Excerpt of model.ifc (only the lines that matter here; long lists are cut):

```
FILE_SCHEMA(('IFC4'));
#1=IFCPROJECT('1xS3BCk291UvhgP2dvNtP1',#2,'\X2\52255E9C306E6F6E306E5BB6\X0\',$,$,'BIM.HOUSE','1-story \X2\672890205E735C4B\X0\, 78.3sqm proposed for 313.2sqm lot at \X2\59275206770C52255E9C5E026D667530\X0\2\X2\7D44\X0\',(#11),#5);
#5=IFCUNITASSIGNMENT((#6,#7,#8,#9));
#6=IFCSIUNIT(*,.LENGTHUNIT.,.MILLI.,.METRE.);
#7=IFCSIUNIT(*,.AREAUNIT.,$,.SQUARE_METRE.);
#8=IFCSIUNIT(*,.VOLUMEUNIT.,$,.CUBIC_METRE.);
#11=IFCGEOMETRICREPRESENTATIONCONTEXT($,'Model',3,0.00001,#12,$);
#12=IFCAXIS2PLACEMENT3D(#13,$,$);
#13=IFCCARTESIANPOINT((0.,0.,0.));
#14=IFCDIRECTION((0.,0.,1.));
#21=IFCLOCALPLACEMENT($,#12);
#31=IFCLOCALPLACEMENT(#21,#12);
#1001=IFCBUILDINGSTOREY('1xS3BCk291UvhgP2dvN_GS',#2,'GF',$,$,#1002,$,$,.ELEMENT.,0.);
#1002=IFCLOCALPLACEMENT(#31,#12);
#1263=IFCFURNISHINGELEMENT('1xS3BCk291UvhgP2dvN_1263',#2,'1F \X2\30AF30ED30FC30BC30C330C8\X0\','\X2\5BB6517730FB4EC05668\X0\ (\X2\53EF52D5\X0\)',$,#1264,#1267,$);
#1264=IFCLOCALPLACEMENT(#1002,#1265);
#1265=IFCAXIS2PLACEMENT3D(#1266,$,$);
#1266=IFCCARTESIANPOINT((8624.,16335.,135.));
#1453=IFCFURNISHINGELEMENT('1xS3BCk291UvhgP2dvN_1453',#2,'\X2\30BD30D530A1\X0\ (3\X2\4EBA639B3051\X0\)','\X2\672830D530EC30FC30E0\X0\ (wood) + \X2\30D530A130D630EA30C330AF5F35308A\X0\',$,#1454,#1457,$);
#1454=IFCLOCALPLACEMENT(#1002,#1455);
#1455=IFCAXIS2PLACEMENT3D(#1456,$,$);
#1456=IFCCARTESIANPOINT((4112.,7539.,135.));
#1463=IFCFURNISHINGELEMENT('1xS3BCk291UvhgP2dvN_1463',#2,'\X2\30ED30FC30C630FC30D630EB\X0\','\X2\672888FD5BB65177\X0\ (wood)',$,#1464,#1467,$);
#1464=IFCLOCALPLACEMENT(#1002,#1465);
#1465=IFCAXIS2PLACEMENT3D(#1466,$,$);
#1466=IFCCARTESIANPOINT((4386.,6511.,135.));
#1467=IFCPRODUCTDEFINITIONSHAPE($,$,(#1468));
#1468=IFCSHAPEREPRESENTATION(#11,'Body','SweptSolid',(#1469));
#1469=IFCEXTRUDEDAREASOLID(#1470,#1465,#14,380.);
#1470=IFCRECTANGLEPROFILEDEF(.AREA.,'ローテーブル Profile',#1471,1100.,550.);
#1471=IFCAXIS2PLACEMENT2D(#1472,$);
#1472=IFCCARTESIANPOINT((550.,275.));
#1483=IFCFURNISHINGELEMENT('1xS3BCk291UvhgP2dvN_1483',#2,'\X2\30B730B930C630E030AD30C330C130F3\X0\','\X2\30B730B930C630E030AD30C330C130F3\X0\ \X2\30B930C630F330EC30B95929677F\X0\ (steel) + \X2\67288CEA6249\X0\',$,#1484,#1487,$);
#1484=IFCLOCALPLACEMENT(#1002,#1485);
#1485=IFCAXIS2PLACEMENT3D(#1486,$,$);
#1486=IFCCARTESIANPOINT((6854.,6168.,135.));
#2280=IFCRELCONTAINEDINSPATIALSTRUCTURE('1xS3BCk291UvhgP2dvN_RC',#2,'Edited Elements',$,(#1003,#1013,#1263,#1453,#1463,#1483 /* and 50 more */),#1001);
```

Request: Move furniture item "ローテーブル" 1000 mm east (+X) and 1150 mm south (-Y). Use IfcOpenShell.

```python
import ifcopenshell
import ifcopenshell.api.geometry
import ifcopenshell.util.placement
import ifcopenshell.util.unit

model = ifcopenshell.open("model.ifc")
unit_scale = ifcopenshell.util.unit.calculate_unit_scale(model)

item = model.by_id(1463)
matrix = ifcopenshell.util.placement.get_local_placement(item.ObjectPlacement)
matrix[0, 3] += 1 / unit_scale
matrix[1, 3] -= 1.15 / unit_scale
ifcopenshell.api.geometry.edit_object_placement(model, product=item, matrix=matrix, is_si=False)

print(ifcopenshell.util.placement.get_local_placement(item.ObjectPlacement).round(3) + 0.0)

model.write("model_updated.ifc")
```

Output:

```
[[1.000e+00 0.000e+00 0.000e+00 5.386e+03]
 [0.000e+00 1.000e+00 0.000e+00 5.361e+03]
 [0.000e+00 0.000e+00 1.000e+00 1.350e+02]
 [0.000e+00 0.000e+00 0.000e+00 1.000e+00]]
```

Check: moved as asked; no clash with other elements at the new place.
